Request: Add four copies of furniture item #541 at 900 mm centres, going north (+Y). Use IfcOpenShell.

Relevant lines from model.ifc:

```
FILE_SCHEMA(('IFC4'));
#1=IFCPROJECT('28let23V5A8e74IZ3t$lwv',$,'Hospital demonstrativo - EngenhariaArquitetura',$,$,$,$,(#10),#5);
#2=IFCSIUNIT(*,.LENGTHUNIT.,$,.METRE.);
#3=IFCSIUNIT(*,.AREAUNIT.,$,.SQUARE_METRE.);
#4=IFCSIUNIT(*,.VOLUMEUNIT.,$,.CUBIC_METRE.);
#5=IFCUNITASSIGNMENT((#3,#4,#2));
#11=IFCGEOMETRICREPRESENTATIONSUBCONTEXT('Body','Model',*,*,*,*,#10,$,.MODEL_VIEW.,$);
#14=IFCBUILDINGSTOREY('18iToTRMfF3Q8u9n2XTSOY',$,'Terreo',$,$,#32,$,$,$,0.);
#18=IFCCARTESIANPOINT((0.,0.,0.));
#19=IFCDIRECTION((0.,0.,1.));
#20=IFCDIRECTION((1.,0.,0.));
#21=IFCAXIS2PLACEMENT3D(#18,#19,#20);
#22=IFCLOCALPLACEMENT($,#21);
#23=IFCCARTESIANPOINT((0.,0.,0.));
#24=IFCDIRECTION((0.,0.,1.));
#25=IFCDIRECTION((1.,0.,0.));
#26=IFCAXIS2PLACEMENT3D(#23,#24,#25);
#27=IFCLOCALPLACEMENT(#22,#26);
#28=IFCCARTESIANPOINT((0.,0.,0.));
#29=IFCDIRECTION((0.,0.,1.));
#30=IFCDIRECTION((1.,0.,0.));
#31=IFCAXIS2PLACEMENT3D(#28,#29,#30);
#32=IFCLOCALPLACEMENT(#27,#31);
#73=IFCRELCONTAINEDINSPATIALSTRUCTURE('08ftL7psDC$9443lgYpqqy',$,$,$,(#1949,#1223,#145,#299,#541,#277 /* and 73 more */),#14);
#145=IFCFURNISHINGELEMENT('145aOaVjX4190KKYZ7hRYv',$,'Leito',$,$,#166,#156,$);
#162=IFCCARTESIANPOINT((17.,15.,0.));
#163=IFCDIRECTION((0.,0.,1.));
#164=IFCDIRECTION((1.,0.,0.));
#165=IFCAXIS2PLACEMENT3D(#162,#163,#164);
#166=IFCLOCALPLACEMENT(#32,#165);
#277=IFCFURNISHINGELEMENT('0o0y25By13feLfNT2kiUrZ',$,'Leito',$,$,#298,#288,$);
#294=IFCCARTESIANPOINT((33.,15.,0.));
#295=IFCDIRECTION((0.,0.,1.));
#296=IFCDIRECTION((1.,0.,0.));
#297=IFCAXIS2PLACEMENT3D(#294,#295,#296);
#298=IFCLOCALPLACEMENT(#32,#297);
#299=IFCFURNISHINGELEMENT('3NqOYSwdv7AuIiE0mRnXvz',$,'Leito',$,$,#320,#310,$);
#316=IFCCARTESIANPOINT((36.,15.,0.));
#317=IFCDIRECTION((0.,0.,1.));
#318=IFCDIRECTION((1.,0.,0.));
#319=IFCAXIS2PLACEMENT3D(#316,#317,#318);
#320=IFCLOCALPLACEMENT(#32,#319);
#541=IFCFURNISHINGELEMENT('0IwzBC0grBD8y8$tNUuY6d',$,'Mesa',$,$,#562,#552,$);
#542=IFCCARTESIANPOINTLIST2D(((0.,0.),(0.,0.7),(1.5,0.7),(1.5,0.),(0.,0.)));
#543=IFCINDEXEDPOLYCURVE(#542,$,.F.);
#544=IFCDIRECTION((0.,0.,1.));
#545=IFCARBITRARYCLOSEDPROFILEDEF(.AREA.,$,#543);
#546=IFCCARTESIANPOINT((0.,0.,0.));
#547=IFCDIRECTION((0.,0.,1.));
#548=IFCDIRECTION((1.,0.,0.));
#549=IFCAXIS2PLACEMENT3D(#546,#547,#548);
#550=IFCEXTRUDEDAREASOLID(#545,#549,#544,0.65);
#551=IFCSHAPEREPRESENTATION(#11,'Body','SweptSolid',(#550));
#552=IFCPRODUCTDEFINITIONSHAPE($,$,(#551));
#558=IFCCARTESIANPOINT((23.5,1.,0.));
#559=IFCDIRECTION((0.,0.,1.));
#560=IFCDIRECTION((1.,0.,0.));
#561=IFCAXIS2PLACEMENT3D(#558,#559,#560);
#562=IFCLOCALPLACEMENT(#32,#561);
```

```python
import numpy as np
import ifcopenshell
import ifcopenshell.api.geometry
import ifcopenshell.api.root
import ifcopenshell.util.element
import ifcopenshell.util.placement
import ifcopenshell.util.unit

model = ifcopenshell.open("model.ifc")
unit_scale = ifcopenshell.util.unit.calculate_unit_scale(model)

source = model.by_guid("0IwzBC0grBD8y8$tNUuY6d")
base = ifcopenshell.util.placement.get_local_placement(source.ObjectPlacement)
step = np.array([0.0, 1.0, 0.0]) * 0.9 / unit_scale

for i in range(1, 5):
    copy = ifcopenshell.api.root.copy_class(model, product=source)
    copy.Representation = ifcopenshell.util.element.copy_deep(
        model, source.Representation, exclude=["IfcGeometricRepresentationContext", "IfcRepresentationMap"]
    )
    matrix = base.copy()
    matrix[:3, 3] += i * step
    print("added at", matrix[:3, 3].round(3) + 0.0)
    ifcopenshell.api.geometry.edit_object_placement(model, product=copy, matrix=matrix, is_si=False)

model.write("model_updated.ifc")
```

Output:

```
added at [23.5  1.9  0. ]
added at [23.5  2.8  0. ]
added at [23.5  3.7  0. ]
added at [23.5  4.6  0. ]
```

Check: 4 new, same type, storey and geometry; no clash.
